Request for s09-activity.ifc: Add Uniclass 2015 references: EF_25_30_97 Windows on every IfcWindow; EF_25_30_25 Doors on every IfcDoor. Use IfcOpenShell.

First a look at what the model holds.

```python
import ifcopenshell

model = ifcopenshell.open("s09-activity.ifc")
print(model.schema)
print("classifications:", [c.Name for c in model.by_type("IfcClassification")])
for ifc_class in ("IfcDoor", "IfcRoof", "IfcStair", "IfcWall", "IfcWindow"):
    print(ifc_class, len(model.by_type(ifc_class)))
```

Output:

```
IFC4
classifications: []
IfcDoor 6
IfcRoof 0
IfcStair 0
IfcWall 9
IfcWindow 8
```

```python
import ifcopenshell
import ifcopenshell.api.classification

model = ifcopenshell.open("s09-activity.ifc")

system = ifcopenshell.api.classification.add_classification(model, classification="Uniclass 2015")

codes = {
    "IfcWindow": ("EF_25_30_97", "Windows"),
    "IfcDoor": ("EF_25_30_25", "Doors"),
}
for ifc_class, (code, name) in codes.items():
    products = model.by_type(ifc_class)
    ifcopenshell.api.classification.add_reference(
        model, products=products, classification=system, identification=code, name=name
    )
    print(code, len(products))

model.write("s09-activity_updated.ifc")
```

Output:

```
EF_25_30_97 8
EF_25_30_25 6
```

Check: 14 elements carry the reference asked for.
